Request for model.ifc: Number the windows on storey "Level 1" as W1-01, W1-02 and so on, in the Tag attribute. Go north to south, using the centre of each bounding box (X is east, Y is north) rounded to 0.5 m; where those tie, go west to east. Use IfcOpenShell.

First a look at what the model holds.

```python
import ifcopenshell
import ifcopenshell.util.element
import ifcopenshell.util.placement

model = ifcopenshell.open("model.ifc")
print(model.schema)
storey = next(s for s in model.by_type("IfcBuildingStorey") if s.Name == "Level 1")
windows = [e for e in ifcopenshell.util.element.get_decomposition(storey) if e.is_a("IfcWindow")]
for e in sorted(windows, key=lambda e: e.id()):
    origin = ifcopenshell.util.placement.get_local_placement(e.ObjectPlacement)[:3, 3]
    print(e.id(), e.Tag, e.Name, origin.round(2) + 0.0, sep=" | ")
```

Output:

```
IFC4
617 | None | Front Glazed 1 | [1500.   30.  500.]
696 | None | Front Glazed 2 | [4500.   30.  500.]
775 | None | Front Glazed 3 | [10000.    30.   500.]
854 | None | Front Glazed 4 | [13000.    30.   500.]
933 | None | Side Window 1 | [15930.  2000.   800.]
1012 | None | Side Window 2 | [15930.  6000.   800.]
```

```python
import ifcopenshell
import ifcopenshell.geom
import ifcopenshell.util.element
import ifcopenshell.util.shape

model = ifcopenshell.open("model.ifc")
settings = ifcopenshell.geom.settings()
settings.set("use-world-coords", True)


def centre(element):
    shape = ifcopenshell.geom.create_shape(settings, element)
    return ifcopenshell.util.shape.get_bbox_centroid(shape.geometry)


storey = next(s for s in model.by_type("IfcBuildingStorey") if s.Name == "Level 1")
windows = [e for e in ifcopenshell.util.element.get_decomposition(storey) if e.is_a("IfcWindow")]

# Insertion points can sit at a corner or the storey origin, so sort by the geometry (in metres).
centres = {e: centre(e) for e in windows}
windows.sort(key=lambda e: (-round(centres[e][1] / 0.5), centres[e][0]))

for i, e in enumerate(windows, start=1):
    number = f"W1-{i:02d}"
    e.Tag = number
    print(e.id(), number)

model.write("model_edited.ifc")
```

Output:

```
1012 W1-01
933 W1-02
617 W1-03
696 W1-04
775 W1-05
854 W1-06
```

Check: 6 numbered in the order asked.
